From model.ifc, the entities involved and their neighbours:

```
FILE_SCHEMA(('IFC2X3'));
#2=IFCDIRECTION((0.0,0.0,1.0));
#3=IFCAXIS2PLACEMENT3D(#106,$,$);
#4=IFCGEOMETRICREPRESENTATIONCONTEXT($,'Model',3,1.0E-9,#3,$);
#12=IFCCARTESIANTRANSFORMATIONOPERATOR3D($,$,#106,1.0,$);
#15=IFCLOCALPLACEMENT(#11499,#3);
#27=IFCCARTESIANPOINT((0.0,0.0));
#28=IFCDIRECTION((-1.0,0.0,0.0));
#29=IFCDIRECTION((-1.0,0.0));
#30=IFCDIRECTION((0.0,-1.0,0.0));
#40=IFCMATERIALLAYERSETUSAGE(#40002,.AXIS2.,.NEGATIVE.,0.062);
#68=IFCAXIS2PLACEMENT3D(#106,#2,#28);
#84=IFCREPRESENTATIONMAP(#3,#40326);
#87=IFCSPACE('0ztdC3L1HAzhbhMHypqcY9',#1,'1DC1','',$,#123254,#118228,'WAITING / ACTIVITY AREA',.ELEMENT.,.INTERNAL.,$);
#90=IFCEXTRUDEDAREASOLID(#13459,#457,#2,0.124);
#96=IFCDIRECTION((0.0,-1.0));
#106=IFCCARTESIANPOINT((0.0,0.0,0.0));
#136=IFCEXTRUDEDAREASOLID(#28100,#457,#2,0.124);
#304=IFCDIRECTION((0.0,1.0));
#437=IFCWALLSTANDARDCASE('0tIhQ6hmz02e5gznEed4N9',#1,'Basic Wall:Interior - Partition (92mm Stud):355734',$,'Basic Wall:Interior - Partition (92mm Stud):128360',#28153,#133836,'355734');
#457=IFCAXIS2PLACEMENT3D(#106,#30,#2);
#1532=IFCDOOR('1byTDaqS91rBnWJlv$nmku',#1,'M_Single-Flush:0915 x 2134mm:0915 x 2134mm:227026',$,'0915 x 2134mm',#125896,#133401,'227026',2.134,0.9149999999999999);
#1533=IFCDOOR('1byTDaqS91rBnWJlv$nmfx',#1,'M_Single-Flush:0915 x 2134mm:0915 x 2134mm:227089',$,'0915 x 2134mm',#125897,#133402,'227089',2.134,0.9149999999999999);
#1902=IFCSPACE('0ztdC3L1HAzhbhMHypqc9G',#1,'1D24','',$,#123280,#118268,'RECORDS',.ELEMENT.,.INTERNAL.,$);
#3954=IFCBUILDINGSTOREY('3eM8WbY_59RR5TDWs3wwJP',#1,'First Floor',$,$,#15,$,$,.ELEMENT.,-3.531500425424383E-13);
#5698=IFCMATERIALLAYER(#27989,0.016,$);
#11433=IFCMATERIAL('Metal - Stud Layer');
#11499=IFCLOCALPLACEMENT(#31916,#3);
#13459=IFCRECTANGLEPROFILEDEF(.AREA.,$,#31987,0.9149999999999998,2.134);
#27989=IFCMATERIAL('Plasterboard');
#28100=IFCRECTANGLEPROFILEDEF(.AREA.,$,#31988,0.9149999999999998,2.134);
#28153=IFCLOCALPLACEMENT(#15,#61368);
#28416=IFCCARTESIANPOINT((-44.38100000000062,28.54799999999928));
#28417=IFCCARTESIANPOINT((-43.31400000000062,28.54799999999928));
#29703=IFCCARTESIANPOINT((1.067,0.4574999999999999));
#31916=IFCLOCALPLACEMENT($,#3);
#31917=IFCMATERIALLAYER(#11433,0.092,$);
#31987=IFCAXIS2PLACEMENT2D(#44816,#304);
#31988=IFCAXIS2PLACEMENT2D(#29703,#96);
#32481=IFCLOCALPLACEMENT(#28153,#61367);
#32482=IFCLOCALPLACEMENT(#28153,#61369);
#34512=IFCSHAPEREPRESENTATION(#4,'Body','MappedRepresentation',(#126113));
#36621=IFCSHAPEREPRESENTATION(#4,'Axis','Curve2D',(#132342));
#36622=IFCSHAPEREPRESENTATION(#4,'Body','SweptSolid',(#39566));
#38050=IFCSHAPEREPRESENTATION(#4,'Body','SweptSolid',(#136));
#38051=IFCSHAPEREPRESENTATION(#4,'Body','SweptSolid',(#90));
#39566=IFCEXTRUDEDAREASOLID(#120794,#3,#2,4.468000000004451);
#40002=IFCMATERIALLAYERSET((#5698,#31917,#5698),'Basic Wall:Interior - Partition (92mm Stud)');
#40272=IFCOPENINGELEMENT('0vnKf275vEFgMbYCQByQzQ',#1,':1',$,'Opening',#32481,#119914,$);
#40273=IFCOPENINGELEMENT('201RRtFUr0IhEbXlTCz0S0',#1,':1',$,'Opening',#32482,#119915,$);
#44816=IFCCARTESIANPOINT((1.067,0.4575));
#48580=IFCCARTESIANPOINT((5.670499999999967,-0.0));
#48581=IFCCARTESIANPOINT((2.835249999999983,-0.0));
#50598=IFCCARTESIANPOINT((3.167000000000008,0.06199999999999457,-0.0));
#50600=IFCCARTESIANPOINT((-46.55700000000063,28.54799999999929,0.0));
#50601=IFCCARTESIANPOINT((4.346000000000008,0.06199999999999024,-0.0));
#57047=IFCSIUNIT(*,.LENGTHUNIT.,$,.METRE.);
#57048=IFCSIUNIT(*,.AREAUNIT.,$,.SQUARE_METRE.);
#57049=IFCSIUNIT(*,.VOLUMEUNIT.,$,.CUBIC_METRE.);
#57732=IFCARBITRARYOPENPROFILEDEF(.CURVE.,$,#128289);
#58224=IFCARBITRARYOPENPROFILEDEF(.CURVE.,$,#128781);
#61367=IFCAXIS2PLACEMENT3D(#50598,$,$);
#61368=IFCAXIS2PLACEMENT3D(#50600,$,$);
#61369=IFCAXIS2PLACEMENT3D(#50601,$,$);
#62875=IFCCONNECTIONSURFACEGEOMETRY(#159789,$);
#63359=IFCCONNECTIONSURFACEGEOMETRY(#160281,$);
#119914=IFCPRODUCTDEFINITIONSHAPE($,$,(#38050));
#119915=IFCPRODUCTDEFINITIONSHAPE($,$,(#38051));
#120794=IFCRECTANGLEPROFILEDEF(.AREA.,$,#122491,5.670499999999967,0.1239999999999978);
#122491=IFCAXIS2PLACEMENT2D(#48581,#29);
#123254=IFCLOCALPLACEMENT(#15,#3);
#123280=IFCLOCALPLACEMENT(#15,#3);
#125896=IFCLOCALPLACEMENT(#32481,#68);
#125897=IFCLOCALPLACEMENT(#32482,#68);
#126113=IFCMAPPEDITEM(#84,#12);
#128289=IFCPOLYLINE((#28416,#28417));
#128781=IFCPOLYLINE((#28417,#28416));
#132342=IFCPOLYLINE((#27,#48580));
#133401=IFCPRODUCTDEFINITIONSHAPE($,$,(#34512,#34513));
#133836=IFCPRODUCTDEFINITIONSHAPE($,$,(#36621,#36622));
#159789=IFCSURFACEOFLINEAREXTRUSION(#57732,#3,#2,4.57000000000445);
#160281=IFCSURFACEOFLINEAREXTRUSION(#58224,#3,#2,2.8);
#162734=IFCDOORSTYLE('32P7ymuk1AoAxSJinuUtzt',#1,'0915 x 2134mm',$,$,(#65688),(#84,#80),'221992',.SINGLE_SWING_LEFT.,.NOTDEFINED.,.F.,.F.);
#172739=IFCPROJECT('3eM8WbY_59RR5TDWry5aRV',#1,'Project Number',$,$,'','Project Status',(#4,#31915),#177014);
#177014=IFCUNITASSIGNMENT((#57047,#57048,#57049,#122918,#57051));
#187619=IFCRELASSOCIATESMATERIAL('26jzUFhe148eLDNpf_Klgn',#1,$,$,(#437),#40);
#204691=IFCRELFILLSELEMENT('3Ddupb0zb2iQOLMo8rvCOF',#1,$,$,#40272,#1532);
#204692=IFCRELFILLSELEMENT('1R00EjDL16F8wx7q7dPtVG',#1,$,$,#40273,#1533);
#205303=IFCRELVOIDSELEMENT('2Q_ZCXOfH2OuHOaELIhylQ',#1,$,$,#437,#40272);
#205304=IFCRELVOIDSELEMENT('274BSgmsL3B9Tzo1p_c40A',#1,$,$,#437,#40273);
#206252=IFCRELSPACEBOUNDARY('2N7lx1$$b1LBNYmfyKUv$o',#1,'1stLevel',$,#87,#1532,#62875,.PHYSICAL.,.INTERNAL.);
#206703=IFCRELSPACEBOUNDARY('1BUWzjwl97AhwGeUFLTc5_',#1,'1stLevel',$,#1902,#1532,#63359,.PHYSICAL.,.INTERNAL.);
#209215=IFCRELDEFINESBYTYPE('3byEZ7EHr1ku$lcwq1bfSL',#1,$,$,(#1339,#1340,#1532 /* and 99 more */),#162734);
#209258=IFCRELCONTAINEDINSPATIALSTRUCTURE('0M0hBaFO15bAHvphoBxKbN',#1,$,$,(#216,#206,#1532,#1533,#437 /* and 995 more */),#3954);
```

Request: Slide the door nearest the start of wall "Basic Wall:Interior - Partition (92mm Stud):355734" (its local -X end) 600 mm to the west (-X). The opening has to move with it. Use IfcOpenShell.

```python
import numpy as np
import ifcopenshell
import ifcopenshell.api.geometry
import ifcopenshell.util.placement

model = ifcopenshell.open("model.ifc")

door = model.by_guid("1byTDaqS91rBnWJlv$nmku")
opening = door.FillsVoids[0].RelatingOpeningElement
wall = opening.VoidsElements[0].RelatingBuildingElement

wall_matrix = ifcopenshell.util.placement.get_local_placement(wall.ObjectPlacement)
shift = wall_matrix[:3, 0] * -0.6
before = ifcopenshell.util.placement.get_local_placement(door.ObjectPlacement)[:3, 3].copy()

# The door is placed relative to its opening, so it follows when the opening moves.
matrix = ifcopenshell.util.placement.get_local_placement(opening.ObjectPlacement)
matrix[:3, 3] += shift
ifcopenshell.api.geometry.edit_object_placement(
    model, product=opening, matrix=matrix, is_si=False, should_transform_children=True
)

# Space boundary surfaces are stored in each space's coordinates; move them too.
for rel in door.ProvidesBoundaries:
    if not rel.ConnectionGeometry:
        continue
    surface = rel.ConnectionGeometry.SurfaceOnRelatingElement
    space_matrix = ifcopenshell.util.placement.get_local_placement(rel.RelatingSpace.ObjectPlacement)
    point = np.array(surface.Position.Location.Coordinates) + space_matrix[:3, :3].T @ shift
    surface.Position = model.createIfcAxis2Placement3D(
        model.createIfcCartesianPoint(point.tolist()), surface.Position.Axis, surface.Position.RefDirection
    )

after = ifcopenshell.util.placement.get_local_placement(door.ObjectPlacement)[:3, 3]
print("door moved by", (after - before).round(3) + 0.0)

model.write("model_updated.ifc")
```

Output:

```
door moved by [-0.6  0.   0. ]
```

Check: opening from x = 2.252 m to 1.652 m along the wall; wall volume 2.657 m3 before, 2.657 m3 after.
